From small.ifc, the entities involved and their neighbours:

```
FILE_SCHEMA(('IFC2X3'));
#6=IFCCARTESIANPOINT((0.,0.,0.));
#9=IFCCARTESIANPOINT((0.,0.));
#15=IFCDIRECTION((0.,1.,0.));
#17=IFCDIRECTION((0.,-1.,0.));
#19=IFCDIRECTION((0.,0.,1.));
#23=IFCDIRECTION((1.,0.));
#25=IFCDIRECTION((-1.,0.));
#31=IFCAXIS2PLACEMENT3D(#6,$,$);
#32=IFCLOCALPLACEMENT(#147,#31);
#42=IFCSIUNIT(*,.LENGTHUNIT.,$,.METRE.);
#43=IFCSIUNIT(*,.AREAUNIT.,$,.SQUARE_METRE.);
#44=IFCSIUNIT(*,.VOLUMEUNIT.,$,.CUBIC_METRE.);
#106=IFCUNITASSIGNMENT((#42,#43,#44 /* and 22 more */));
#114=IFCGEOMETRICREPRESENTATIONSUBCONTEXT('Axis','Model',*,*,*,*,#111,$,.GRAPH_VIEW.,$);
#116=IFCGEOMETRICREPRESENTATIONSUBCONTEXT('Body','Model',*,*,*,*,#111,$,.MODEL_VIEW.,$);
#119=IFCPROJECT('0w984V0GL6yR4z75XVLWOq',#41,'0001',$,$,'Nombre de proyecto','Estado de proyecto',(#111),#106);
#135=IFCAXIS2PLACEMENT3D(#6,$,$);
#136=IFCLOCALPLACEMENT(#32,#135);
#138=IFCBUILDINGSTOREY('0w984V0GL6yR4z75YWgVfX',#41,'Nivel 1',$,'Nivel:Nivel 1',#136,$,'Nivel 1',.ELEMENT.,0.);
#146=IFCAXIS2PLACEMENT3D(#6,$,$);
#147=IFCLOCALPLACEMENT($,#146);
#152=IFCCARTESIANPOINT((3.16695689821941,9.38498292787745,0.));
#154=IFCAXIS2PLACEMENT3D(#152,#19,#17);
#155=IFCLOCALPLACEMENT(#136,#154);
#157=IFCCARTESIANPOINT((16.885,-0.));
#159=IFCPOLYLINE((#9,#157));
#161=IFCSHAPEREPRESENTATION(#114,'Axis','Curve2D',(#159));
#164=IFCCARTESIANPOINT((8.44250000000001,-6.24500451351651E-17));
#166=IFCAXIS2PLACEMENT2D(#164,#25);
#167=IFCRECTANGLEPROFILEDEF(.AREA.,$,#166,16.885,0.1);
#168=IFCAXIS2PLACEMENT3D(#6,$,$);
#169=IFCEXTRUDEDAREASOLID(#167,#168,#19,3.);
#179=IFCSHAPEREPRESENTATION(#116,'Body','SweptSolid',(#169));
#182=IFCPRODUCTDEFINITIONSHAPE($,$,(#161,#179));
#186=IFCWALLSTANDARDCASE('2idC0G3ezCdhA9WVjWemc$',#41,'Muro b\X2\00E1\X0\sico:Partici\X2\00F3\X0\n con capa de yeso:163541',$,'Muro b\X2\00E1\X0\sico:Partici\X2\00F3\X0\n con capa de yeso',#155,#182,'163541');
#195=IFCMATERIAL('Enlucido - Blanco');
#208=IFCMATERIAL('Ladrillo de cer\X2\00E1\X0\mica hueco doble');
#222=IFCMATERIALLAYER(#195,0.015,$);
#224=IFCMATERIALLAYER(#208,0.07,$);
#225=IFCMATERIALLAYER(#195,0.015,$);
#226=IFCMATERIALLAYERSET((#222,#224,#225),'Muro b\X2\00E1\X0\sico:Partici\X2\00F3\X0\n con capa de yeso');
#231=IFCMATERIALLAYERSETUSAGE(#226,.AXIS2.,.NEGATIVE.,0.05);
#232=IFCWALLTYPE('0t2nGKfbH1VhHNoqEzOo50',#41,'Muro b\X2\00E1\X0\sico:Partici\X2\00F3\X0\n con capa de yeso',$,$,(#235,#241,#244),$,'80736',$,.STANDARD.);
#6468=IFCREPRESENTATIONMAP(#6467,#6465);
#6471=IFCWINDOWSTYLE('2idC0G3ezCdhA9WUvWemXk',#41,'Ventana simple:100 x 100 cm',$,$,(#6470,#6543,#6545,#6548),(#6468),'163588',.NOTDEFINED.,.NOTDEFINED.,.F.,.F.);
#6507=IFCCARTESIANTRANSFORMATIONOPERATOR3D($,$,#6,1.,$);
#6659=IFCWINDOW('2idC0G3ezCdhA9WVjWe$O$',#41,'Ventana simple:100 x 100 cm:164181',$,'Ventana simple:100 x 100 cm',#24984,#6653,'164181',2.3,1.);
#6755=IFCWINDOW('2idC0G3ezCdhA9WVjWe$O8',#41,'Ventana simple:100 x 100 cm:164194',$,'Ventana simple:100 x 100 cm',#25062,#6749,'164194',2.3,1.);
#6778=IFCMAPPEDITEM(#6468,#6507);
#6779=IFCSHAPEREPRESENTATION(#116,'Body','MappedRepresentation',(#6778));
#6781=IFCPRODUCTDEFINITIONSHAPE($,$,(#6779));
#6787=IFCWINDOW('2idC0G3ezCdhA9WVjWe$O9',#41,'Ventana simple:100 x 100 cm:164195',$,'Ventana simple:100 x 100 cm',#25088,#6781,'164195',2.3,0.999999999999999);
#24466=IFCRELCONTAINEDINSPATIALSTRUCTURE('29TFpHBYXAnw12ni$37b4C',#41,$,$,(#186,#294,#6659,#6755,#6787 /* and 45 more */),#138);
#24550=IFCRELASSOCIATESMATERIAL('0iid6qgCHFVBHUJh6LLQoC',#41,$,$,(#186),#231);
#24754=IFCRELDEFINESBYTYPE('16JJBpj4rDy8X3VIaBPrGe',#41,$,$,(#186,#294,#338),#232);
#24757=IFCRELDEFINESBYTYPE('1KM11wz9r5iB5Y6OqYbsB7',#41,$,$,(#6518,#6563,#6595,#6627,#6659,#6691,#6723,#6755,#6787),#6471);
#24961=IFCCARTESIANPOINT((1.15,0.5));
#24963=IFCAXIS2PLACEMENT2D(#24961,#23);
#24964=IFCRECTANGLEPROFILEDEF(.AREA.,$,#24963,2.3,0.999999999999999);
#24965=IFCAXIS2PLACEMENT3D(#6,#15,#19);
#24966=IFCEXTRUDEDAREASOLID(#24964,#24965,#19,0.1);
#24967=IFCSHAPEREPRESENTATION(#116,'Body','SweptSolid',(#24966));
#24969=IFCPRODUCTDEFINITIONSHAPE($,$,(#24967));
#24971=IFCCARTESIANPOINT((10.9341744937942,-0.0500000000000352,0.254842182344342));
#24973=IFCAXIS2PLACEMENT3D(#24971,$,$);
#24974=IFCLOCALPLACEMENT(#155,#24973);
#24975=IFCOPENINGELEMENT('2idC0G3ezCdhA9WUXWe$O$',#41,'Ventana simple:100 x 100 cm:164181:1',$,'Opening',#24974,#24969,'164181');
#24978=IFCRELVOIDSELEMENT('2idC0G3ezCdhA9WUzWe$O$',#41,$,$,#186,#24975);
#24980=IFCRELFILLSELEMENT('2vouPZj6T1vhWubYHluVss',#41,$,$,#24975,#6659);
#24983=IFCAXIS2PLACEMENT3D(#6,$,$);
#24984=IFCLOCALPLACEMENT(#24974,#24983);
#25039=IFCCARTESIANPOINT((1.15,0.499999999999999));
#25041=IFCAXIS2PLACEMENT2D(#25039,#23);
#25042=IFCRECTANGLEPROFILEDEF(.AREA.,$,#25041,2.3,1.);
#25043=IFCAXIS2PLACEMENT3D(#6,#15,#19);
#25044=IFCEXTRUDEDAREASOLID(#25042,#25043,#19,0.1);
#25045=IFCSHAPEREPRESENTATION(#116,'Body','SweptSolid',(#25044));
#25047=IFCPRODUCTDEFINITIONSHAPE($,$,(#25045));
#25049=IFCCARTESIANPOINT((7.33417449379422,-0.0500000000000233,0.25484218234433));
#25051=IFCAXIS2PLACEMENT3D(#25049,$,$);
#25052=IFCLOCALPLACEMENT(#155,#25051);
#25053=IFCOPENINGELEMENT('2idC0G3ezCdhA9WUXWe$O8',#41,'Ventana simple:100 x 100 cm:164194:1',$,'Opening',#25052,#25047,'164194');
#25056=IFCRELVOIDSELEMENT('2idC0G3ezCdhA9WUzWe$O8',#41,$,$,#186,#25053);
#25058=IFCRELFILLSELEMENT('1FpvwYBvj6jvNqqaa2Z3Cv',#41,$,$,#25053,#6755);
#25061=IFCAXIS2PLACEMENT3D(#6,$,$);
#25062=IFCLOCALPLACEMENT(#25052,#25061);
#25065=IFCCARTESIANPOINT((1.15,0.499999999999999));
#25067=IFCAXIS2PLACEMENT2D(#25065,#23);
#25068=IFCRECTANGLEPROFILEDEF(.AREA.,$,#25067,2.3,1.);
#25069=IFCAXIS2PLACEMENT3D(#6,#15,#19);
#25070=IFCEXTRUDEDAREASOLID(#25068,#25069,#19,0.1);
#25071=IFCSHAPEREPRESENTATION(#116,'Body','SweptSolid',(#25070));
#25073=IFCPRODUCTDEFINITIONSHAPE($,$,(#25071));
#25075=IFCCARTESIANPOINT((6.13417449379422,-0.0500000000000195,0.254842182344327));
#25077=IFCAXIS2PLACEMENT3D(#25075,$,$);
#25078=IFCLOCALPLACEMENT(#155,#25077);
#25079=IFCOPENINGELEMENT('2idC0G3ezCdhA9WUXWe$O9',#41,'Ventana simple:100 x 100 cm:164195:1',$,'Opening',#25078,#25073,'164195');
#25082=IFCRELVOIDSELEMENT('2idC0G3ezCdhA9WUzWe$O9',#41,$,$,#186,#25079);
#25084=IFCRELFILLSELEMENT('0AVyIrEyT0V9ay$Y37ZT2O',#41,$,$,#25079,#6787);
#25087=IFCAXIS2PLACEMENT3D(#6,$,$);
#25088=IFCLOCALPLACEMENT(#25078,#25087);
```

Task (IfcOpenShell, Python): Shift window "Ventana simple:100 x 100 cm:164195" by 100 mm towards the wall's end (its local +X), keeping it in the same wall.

```python
import ifcopenshell
import ifcopenshell.api.geometry
import ifcopenshell.util.placement
import ifcopenshell.util.unit

model = ifcopenshell.open("small.ifc")
unit_scale = ifcopenshell.util.unit.calculate_unit_scale(model)

window = model.by_guid("2idC0G3ezCdhA9WVjWe$O9")
opening = window.FillsVoids[0].RelatingOpeningElement
wall = opening.VoidsElements[0].RelatingBuildingElement

wall_matrix = ifcopenshell.util.placement.get_local_placement(wall.ObjectPlacement)
shift = wall_matrix[:3, 0] * 0.1 / unit_scale
before = ifcopenshell.util.placement.get_local_placement(window.ObjectPlacement)[:3, 3].copy()

# The window is placed relative to its opening, so it follows when the opening moves.
matrix = ifcopenshell.util.placement.get_local_placement(opening.ObjectPlacement)
matrix[:3, 3] += shift
ifcopenshell.api.geometry.edit_object_placement(
    model, product=opening, matrix=matrix, is_si=False, should_transform_children=True
)

after = ifcopenshell.util.placement.get_local_placement(window.ObjectPlacement)[:3, 3]
print("window moved by", (after - before).round(3) + 0.0)

model.write("small-out.ifc")
```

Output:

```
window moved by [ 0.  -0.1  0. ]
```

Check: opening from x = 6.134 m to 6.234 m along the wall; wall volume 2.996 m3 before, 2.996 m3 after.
